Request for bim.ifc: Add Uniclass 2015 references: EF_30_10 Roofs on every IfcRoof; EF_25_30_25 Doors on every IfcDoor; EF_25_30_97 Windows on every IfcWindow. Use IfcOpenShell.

First a look at what the model holds.

```python
import ifcopenshell

model = ifcopenshell.open("bim.ifc")
print(model.schema)
print("classifications:", [c.Name for c in model.by_type("IfcClassification")])
for ifc_class in ("IfcDoor", "IfcRoof", "IfcStair", "IfcWall", "IfcWindow"):
    print(ifc_class, len(model.by_type(ifc_class)))
```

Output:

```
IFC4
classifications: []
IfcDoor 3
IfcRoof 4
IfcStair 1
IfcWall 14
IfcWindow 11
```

```python
import ifcopenshell
import ifcopenshell.api.classification

model = ifcopenshell.open("bim.ifc")

system = ifcopenshell.api.classification.add_classification(model, classification="Uniclass 2015")

codes = {
    "IfcRoof": ("EF_30_10", "Roofs"),
    "IfcDoor": ("EF_25_30_25", "Doors"),
    "IfcWindow": ("EF_25_30_97", "Windows"),
}
for ifc_class, (code, name) in codes.items():
    products = model.by_type(ifc_class)
    ifcopenshell.api.classification.add_reference(
        model, products=products, classification=system, identification=code, name=name
    )
    print(code, len(products))

model.write("bim_updated.ifc")
```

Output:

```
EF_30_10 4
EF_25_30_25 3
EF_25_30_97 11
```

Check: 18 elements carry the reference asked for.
